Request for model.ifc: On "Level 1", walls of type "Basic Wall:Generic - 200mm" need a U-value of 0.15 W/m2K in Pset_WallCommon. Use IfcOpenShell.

First a look at what the model holds.

```python
import ifcopenshell
import ifcopenshell.util.element

model = ifcopenshell.open("model.ifc")
print(model.schema)
storey = next(s for s in model.by_type("IfcBuildingStorey") if s.Name == "Level 1")
walls = [e for e in ifcopenshell.util.element.get_decomposition(storey) if e.is_a("IfcWall")]
seen = {}
for e in walls:
    element_type = ifcopenshell.util.element.get_type(e)
    key = (element_type.Name if element_type != e and element_type else None, ifcopenshell.util.element.get_pset(e, "Pset_WallCommon", "ThermalTransmittance"))
    seen[key] = seen.get(key, 0) + 1
for (name, value), count in sorted(seen.items(), key=str):
    print(count, "x", name, "|", value)
```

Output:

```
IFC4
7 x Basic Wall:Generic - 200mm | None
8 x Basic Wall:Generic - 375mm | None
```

```python
import ifcopenshell
import ifcopenshell.api.pset
import ifcopenshell.util.element

model = ifcopenshell.open("model.ifc")

storey = next(s for s in model.by_type("IfcBuildingStorey") if s.Name == "Level 1")
walls = [e for e in ifcopenshell.util.element.get_decomposition(storey) if e.is_a("IfcWall")]

count = 0
for e in walls:
    element_type = ifcopenshell.util.element.get_type(e)
    if element_type in (None, e) or element_type.Name != "Basic Wall:Generic - 200mm":
        continue
    # add_pset returns the element's existing set when there is one.
    pset = ifcopenshell.api.pset.add_pset(model, product=e, name="Pset_WallCommon")
    ifcopenshell.api.pset.edit_pset(model, pset=pset, properties={"ThermalTransmittance": 0.15})
    count += 1

print(count, "walls updated")

model.write("model_edited.ifc")
```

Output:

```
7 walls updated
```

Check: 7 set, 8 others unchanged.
